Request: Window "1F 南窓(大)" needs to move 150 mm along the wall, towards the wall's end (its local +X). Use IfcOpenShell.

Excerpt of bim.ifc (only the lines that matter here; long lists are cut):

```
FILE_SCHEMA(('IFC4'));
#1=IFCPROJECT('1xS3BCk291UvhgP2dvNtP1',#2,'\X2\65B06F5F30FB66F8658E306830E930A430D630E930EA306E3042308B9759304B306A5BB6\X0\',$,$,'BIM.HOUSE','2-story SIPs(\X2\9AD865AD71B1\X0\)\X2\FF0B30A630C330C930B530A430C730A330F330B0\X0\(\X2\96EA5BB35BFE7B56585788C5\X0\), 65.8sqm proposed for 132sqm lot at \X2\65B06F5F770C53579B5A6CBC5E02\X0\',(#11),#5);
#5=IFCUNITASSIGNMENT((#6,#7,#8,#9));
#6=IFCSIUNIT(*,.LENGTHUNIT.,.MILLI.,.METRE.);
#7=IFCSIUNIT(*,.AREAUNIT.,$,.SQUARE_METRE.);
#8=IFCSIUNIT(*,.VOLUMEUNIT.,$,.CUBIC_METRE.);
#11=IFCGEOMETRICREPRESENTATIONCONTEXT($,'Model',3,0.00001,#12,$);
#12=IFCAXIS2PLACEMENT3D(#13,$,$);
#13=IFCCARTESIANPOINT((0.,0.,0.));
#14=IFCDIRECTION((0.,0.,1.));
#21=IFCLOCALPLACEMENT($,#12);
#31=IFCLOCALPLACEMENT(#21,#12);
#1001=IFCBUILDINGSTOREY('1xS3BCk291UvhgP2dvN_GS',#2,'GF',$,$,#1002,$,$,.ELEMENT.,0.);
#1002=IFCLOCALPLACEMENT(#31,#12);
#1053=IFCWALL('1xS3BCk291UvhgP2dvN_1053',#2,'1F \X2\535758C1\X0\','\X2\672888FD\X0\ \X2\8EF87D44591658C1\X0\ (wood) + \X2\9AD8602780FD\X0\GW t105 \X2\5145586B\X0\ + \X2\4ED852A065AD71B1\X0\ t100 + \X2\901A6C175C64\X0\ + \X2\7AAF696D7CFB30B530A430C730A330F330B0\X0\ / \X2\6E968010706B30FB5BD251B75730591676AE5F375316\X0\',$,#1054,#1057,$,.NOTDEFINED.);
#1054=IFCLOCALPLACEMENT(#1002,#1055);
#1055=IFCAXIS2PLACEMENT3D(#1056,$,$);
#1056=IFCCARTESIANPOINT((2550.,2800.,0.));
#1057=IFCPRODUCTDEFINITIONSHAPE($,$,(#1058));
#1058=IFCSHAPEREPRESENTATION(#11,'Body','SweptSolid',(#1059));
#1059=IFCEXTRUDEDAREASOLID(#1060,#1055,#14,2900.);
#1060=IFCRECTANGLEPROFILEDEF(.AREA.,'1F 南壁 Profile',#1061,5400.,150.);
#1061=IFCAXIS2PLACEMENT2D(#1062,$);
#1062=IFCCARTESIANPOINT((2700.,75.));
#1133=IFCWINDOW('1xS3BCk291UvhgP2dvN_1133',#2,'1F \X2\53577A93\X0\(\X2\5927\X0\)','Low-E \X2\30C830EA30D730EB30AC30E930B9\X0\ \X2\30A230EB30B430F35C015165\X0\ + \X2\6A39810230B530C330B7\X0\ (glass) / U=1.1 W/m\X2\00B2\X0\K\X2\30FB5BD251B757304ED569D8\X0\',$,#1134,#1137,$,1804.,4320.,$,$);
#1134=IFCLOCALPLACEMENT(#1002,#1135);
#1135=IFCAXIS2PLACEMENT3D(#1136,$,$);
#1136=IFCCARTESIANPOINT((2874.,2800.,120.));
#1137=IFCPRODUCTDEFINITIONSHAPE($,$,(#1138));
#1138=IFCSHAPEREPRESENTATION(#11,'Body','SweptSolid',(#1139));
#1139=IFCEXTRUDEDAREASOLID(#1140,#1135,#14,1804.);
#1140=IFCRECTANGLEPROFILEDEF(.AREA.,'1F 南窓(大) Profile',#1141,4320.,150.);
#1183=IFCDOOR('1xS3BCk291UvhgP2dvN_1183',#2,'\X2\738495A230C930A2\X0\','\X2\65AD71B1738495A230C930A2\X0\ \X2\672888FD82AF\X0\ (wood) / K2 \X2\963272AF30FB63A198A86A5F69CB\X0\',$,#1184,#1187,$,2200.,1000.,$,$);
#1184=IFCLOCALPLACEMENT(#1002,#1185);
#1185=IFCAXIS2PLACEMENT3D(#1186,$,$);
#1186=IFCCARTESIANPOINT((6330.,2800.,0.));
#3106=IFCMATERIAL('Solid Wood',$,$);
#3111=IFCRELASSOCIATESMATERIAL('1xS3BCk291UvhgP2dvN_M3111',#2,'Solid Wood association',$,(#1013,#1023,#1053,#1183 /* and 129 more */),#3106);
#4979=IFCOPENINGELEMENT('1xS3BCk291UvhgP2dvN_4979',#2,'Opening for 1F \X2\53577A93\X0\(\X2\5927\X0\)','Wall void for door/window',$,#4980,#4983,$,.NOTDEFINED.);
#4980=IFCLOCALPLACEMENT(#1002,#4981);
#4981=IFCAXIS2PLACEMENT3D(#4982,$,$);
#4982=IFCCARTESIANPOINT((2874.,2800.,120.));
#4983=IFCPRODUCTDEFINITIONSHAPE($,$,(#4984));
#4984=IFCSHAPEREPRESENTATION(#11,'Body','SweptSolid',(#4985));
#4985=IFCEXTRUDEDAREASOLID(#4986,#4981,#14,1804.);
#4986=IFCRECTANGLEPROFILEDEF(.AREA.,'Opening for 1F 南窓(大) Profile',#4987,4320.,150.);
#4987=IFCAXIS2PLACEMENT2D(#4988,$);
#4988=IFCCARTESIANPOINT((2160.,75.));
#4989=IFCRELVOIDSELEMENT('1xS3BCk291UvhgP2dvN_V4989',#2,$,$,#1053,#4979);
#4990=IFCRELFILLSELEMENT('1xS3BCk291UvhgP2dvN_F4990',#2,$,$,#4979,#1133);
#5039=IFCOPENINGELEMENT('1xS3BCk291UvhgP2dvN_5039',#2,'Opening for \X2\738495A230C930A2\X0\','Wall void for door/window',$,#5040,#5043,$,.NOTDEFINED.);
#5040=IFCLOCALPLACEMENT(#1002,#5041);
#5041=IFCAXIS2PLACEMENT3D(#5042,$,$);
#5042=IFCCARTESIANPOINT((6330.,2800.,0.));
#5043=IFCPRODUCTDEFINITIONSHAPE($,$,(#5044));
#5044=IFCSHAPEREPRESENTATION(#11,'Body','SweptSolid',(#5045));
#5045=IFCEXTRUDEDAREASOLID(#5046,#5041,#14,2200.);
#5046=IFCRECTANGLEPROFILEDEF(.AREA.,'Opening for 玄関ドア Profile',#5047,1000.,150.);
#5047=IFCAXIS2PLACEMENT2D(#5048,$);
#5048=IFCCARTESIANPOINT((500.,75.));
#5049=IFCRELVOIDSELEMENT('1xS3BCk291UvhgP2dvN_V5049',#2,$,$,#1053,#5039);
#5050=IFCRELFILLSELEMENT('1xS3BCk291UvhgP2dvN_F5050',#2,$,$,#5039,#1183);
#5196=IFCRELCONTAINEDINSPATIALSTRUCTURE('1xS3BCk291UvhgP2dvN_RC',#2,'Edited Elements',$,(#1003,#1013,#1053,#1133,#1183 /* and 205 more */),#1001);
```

```python
import ifcopenshell
import ifcopenshell.api.geometry
import ifcopenshell.util.placement

model = ifcopenshell.open("bim.ifc")

window = model.by_guid("1xS3BCk291UvhgP2dvN_1133")
opening = window.FillsVoids[0].RelatingOpeningElement
wall = opening.VoidsElements[0].RelatingBuildingElement

wall_matrix = ifcopenshell.util.placement.get_local_placement(wall.ObjectPlacement)
shift = wall_matrix[:3, 0] * 150.0
before = ifcopenshell.util.placement.get_local_placement(window.ObjectPlacement)[:3, 3].copy()

# The window is not placed relative to its opening, so move both.
for product in (opening, window):
    matrix = ifcopenshell.util.placement.get_local_placement(product.ObjectPlacement)
    matrix[:3, 3] += shift
    ifcopenshell.api.geometry.edit_object_placement(model, product=product, matrix=matrix, is_si=False)

after = ifcopenshell.util.placement.get_local_placement(window.ObjectPlacement)[:3, 3]
print("window moved by", (after - before).round(3) + 0.0)

model.write("bim-out.ifc")
```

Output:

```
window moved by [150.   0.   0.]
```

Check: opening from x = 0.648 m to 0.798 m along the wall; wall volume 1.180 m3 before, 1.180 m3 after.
